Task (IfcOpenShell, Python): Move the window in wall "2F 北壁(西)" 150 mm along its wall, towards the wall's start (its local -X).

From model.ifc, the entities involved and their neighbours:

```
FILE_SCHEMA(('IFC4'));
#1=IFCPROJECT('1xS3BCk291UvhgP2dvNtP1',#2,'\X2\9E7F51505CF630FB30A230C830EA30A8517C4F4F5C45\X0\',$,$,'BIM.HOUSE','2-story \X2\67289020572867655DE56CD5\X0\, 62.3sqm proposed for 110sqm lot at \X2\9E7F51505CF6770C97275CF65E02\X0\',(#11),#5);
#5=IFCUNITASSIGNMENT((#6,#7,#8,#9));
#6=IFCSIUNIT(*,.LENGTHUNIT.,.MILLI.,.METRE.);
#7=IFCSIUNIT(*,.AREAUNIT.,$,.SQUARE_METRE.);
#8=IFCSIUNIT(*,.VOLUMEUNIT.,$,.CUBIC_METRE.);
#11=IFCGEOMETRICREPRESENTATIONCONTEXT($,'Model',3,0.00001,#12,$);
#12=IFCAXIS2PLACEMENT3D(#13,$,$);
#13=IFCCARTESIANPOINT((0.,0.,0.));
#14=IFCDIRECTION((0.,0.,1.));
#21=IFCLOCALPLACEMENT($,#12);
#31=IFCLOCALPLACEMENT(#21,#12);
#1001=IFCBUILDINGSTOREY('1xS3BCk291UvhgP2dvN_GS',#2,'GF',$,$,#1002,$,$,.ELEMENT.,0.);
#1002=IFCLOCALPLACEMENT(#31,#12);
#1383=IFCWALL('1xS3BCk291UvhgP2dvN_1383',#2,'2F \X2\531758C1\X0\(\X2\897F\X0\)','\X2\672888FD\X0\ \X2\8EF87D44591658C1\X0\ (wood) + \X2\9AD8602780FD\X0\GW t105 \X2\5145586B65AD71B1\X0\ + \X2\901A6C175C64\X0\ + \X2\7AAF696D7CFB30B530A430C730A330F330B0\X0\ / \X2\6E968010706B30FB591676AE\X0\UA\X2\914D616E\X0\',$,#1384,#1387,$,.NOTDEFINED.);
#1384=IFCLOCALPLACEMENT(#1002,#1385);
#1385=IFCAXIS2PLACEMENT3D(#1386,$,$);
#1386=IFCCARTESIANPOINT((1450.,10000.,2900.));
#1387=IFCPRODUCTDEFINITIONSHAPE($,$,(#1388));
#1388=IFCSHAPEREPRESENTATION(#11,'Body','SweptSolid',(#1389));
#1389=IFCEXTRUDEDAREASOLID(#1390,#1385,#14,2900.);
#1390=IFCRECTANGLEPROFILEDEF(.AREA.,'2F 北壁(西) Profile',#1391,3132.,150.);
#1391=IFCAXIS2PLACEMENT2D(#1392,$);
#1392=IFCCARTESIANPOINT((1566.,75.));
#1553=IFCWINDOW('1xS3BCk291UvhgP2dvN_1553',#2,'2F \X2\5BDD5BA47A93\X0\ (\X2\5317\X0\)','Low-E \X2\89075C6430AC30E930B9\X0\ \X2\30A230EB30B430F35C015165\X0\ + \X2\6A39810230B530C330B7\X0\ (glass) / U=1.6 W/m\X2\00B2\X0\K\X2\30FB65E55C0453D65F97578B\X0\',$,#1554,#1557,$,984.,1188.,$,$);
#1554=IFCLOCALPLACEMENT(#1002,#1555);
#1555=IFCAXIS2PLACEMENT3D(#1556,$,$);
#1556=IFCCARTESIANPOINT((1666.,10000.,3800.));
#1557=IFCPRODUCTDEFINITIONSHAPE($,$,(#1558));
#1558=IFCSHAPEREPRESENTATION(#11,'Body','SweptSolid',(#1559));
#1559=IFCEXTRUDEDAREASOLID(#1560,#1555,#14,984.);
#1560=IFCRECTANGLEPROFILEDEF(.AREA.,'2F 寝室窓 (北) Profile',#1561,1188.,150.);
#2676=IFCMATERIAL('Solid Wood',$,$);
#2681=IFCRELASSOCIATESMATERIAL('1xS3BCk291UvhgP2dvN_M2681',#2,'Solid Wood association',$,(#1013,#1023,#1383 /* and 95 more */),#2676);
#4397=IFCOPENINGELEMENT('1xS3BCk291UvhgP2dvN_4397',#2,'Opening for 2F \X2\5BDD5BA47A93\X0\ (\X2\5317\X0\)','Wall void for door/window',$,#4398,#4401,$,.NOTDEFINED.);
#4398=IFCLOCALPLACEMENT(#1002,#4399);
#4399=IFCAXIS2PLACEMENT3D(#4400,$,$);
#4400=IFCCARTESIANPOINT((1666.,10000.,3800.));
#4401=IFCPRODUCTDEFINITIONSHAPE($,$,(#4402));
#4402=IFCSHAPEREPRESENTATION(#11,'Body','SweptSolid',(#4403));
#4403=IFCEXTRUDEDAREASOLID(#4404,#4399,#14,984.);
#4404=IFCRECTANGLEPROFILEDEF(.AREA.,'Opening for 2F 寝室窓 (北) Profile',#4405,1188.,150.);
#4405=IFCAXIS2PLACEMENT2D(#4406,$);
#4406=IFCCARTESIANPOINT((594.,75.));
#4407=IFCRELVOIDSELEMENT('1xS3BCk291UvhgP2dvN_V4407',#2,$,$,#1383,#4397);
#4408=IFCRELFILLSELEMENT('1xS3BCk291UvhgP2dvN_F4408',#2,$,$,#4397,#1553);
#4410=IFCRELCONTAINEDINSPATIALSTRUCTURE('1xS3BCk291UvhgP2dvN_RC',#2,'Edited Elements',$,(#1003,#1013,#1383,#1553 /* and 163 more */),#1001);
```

```python
import ifcopenshell
import ifcopenshell.api.geometry
import ifcopenshell.util.placement

model = ifcopenshell.open("model.ifc")

window = model.by_guid("1xS3BCk291UvhgP2dvN_1553")
opening = window.FillsVoids[0].RelatingOpeningElement
wall = opening.VoidsElements[0].RelatingBuildingElement

wall_matrix = ifcopenshell.util.placement.get_local_placement(wall.ObjectPlacement)
shift = wall_matrix[:3, 0] * -150.0
before = ifcopenshell.util.placement.get_local_placement(window.ObjectPlacement)[:3, 3].copy()

# The window is not placed relative to its opening, so move both.
for product in (opening, window):
    matrix = ifcopenshell.util.placement.get_local_placement(product.ObjectPlacement)
    matrix[:3, 3] += shift
    ifcopenshell.api.geometry.edit_object_placement(model, product=product, matrix=matrix, is_si=False)

after = ifcopenshell.util.placement.get_local_placement(window.ObjectPlacement)[:3, 3]
print("window moved by", (after - before).round(3) + 0.0)

model.write("model-out.ifc")
```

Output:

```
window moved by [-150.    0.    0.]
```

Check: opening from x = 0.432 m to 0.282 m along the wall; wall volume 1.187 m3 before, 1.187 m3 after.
